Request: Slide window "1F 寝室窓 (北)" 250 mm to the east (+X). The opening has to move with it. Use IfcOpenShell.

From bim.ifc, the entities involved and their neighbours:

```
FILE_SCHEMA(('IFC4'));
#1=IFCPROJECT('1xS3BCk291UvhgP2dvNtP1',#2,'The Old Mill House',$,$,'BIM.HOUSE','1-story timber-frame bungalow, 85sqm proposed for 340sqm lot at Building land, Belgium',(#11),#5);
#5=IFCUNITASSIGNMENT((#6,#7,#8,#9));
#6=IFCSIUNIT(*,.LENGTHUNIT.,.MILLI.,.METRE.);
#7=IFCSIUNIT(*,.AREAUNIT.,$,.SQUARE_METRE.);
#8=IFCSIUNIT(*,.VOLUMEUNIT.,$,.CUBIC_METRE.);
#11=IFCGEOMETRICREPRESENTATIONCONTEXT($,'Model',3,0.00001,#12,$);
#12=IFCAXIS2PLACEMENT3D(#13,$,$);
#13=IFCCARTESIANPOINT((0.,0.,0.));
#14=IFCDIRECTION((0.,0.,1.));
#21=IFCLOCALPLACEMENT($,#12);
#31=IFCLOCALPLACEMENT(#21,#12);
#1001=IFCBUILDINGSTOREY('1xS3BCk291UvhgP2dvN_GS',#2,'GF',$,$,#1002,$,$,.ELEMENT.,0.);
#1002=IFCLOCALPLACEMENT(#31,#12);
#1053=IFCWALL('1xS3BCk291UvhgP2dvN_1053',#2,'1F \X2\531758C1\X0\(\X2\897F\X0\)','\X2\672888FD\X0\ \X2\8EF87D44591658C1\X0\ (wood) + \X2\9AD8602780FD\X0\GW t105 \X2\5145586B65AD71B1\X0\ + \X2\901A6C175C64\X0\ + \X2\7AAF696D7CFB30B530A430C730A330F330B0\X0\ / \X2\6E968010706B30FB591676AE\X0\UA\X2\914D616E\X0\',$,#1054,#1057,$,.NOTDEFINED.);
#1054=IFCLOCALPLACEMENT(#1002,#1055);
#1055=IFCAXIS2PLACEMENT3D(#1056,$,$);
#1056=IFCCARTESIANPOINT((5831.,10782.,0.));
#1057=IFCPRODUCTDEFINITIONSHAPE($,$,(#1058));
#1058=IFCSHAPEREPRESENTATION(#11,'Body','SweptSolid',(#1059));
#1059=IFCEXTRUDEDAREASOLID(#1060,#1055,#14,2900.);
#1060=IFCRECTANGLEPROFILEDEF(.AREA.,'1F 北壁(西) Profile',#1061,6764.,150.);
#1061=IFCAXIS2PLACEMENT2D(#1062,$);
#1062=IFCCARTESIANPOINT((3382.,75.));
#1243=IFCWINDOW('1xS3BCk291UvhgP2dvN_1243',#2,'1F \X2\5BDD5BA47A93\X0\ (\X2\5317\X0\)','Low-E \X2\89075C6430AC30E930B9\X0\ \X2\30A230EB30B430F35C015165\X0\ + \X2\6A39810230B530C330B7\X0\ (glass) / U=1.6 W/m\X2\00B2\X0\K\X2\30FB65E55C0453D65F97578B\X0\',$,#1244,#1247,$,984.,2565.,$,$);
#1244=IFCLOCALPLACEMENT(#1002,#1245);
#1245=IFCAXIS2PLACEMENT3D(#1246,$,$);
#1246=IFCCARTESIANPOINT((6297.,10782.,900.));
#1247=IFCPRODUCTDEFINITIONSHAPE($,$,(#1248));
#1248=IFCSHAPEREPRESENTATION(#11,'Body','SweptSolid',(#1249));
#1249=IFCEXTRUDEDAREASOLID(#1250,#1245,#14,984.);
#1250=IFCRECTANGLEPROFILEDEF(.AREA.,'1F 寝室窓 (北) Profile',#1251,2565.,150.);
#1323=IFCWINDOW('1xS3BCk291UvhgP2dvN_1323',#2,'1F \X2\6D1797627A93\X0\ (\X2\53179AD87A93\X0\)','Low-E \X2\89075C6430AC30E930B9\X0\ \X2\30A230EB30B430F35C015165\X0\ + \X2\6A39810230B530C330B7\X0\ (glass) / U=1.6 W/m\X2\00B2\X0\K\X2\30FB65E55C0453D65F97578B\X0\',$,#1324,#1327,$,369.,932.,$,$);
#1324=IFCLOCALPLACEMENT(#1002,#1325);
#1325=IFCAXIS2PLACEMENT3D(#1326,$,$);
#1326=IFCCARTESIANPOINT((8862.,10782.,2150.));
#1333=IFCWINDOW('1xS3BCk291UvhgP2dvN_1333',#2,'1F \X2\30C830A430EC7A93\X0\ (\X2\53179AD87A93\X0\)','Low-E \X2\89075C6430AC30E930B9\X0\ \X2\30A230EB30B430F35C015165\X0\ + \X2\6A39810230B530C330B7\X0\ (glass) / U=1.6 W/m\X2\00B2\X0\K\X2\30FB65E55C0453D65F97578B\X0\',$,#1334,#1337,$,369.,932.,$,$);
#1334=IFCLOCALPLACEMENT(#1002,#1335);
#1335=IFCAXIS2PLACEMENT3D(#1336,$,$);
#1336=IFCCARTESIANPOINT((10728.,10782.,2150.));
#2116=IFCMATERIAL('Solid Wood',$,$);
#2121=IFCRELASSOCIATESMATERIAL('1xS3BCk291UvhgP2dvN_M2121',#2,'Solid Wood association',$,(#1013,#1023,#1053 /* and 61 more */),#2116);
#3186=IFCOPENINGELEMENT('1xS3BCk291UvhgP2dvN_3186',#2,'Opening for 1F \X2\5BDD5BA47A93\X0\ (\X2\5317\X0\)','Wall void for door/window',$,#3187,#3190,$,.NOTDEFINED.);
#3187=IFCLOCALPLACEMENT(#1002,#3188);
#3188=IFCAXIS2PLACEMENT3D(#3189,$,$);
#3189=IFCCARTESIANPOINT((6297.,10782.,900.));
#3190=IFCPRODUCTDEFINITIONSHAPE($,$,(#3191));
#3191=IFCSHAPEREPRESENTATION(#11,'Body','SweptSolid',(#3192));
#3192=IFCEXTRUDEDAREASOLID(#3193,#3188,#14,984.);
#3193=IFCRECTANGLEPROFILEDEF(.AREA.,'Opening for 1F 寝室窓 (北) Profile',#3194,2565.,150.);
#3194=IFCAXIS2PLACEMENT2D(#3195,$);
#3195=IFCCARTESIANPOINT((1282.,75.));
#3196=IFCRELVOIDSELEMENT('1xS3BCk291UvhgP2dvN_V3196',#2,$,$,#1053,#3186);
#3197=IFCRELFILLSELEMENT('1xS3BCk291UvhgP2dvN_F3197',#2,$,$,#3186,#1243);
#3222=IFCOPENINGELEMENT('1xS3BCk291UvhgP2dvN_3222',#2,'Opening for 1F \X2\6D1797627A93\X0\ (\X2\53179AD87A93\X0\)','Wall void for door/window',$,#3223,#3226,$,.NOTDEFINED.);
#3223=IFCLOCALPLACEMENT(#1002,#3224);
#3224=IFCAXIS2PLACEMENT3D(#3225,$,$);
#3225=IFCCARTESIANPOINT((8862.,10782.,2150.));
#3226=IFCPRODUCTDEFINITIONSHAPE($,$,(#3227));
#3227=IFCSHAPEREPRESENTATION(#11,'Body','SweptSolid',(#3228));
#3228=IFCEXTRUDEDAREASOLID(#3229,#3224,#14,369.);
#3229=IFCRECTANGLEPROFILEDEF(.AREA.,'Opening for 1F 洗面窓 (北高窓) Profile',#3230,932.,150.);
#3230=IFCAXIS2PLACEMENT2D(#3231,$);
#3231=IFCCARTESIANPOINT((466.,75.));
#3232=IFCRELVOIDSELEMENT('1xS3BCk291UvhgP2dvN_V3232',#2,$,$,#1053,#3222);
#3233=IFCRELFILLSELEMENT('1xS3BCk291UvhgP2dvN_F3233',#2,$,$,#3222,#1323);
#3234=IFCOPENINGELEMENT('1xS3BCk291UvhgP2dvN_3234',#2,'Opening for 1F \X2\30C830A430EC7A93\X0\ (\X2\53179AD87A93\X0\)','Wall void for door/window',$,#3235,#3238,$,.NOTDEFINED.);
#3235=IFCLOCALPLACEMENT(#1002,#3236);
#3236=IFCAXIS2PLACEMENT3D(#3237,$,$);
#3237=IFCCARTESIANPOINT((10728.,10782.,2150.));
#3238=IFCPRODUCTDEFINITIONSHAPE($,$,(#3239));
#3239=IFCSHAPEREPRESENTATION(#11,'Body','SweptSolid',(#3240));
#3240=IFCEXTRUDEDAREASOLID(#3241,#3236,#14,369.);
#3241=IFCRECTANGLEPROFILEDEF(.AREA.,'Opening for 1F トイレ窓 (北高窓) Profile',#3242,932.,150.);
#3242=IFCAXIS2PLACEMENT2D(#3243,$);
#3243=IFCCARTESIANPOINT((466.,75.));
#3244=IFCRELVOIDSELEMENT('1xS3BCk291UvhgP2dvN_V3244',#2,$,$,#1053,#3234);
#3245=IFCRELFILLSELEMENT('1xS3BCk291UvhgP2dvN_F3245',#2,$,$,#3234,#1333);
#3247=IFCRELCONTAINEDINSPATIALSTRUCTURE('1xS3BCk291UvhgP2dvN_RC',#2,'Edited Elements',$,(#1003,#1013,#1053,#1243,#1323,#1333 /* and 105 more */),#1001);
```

```python
import ifcopenshell
import ifcopenshell.api.geometry
import ifcopenshell.util.placement
import ifcopenshell.util.unit

model = ifcopenshell.open("bim.ifc")
unit_scale = ifcopenshell.util.unit.calculate_unit_scale(model)

window = model.by_id(1243)
opening = window.FillsVoids[0].RelatingOpeningElement
wall = opening.VoidsElements[0].RelatingBuildingElement

wall_matrix = ifcopenshell.util.placement.get_local_placement(wall.ObjectPlacement)
shift = wall_matrix[:3, 0] * 0.25 / unit_scale
before = ifcopenshell.util.placement.get_local_placement(window.ObjectPlacement)[:3, 3].copy()

# The window is not placed relative to its opening, so move both.
for product in (opening, window):
    matrix = ifcopenshell.util.placement.get_local_placement(product.ObjectPlacement)
    matrix[:3, 3] += shift
    ifcopenshell.api.geometry.edit_object_placement(model, product=product, matrix=matrix, is_si=False)

after = ifcopenshell.util.placement.get_local_placement(window.ObjectPlacement)[:3, 3]
print("window moved by", (after - before).round(3) + 0.0)

model.write("bim-out.ifc")
```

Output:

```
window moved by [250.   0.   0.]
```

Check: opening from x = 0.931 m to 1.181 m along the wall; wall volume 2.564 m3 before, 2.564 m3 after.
